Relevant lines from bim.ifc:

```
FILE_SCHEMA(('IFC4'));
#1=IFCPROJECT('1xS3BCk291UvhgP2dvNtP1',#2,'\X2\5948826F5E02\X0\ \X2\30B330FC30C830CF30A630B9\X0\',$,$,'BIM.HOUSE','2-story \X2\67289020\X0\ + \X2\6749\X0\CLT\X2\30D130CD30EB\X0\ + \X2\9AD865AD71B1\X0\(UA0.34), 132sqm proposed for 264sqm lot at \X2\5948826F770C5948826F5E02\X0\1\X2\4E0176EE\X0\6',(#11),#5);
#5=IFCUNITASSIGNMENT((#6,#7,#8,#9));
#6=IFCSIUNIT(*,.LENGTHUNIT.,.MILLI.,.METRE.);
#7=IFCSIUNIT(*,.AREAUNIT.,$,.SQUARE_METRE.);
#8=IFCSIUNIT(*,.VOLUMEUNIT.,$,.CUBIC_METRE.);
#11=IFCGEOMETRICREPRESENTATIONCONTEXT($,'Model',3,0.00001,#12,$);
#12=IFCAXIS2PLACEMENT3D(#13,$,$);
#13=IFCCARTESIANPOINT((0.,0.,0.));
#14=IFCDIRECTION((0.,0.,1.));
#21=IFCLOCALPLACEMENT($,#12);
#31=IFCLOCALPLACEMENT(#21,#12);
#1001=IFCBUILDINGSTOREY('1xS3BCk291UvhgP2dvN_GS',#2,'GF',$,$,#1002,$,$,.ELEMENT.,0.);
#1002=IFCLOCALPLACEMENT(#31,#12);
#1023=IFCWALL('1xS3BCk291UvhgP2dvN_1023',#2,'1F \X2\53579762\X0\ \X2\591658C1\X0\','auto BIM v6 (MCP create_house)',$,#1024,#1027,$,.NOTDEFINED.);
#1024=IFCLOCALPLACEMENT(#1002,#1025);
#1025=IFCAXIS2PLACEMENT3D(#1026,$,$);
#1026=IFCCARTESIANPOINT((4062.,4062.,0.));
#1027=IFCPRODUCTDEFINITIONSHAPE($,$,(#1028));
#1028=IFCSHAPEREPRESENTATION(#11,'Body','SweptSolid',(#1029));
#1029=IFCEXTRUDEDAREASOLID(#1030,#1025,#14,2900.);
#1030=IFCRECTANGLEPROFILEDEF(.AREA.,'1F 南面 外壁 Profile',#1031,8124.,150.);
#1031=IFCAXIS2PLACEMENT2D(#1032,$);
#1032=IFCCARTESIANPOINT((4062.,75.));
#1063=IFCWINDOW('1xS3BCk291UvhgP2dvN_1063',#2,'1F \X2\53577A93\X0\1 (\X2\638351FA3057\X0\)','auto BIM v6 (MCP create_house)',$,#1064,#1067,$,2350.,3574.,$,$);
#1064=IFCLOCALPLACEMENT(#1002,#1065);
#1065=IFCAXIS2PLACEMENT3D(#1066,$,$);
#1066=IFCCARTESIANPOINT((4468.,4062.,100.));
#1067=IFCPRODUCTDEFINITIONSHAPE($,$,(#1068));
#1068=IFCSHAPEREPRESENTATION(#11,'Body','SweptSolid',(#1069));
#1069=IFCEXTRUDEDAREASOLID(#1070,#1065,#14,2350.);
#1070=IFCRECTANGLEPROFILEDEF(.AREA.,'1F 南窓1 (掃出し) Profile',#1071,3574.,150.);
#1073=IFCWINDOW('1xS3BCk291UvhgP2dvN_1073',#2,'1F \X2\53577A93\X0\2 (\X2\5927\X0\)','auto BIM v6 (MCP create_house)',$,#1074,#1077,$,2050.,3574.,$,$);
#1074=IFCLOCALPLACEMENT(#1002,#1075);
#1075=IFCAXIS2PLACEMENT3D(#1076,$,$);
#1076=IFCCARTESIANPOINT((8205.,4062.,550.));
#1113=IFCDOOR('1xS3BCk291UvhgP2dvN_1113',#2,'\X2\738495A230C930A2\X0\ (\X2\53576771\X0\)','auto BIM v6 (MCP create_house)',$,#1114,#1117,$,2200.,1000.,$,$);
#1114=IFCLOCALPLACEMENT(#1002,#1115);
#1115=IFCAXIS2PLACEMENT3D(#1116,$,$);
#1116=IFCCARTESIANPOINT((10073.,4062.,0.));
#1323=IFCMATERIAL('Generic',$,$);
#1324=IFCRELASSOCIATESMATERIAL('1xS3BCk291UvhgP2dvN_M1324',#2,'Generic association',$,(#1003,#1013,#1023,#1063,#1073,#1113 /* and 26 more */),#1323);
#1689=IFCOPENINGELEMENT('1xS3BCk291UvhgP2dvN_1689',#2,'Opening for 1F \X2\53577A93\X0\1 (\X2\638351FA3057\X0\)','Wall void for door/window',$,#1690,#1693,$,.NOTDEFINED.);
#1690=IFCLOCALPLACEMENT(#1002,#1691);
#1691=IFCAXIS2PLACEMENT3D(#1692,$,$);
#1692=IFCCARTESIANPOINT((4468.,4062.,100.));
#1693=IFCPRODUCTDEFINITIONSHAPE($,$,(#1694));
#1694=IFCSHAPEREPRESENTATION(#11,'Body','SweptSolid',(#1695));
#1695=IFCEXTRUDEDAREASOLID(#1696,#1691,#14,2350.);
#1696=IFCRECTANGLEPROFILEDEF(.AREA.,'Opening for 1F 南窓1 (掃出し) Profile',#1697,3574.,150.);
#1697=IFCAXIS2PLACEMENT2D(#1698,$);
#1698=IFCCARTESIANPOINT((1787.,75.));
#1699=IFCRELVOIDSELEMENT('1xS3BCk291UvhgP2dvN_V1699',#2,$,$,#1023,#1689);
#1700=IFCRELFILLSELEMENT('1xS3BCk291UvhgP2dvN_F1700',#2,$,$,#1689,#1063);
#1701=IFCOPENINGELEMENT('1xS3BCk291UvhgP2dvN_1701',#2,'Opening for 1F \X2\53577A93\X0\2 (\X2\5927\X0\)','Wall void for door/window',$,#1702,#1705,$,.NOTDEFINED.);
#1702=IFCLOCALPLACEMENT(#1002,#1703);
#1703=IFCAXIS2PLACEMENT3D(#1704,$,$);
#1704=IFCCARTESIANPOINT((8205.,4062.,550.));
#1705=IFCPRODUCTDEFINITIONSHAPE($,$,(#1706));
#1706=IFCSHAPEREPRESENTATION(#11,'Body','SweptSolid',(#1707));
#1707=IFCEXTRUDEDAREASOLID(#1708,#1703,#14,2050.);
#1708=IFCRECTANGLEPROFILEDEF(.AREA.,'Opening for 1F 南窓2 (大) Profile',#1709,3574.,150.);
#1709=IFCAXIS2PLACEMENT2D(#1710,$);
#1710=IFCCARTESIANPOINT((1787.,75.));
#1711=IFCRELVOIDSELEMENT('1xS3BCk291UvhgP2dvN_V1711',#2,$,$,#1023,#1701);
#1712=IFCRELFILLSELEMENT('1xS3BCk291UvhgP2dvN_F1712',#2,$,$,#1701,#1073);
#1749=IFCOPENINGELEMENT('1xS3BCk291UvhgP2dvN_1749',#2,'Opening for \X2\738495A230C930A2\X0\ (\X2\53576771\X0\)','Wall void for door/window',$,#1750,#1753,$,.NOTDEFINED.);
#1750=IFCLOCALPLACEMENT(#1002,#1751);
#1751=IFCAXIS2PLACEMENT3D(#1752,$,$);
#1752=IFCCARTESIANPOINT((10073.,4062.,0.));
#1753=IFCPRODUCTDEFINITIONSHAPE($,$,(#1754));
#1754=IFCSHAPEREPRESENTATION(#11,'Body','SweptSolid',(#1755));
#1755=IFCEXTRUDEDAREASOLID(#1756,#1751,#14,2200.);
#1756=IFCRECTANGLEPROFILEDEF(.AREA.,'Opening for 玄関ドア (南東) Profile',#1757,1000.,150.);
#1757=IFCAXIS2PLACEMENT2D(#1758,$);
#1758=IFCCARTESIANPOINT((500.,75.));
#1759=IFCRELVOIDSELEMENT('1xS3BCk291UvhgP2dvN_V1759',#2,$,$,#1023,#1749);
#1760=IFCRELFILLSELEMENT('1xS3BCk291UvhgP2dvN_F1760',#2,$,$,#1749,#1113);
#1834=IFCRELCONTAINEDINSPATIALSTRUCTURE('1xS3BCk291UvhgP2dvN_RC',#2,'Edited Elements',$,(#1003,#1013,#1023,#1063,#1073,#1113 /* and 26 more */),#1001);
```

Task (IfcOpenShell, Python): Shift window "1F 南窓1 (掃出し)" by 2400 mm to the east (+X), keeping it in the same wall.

```python
import ifcopenshell
import ifcopenshell.api.geometry
import ifcopenshell.util.placement
import ifcopenshell.util.unit

model = ifcopenshell.open("bim.ifc")
unit_scale = ifcopenshell.util.unit.calculate_unit_scale(model)

window = model.by_guid("1xS3BCk291UvhgP2dvN_1063")
opening = window.FillsVoids[0].RelatingOpeningElement
wall = opening.VoidsElements[0].RelatingBuildingElement

wall_matrix = ifcopenshell.util.placement.get_local_placement(wall.ObjectPlacement)
shift = wall_matrix[:3, 0] * 2.4 / unit_scale
before = ifcopenshell.util.placement.get_local_placement(window.ObjectPlacement)[:3, 3].copy()

# The window is not placed relative to its opening, so move both.
for product in (opening, window):
    matrix = ifcopenshell.util.placement.get_local_placement(product.ObjectPlacement)
    matrix[:3, 3] += shift
    ifcopenshell.api.geometry.edit_object_placement(model, product=product, matrix=matrix, is_si=False)

after = ifcopenshell.util.placement.get_local_placement(window.ObjectPlacement)[:3, 3]
print("window moved by", (after - before).round(3) + 0.0)

model.write("bim_v2.ifc")
```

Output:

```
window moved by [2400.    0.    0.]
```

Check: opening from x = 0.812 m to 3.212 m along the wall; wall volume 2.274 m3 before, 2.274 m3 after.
